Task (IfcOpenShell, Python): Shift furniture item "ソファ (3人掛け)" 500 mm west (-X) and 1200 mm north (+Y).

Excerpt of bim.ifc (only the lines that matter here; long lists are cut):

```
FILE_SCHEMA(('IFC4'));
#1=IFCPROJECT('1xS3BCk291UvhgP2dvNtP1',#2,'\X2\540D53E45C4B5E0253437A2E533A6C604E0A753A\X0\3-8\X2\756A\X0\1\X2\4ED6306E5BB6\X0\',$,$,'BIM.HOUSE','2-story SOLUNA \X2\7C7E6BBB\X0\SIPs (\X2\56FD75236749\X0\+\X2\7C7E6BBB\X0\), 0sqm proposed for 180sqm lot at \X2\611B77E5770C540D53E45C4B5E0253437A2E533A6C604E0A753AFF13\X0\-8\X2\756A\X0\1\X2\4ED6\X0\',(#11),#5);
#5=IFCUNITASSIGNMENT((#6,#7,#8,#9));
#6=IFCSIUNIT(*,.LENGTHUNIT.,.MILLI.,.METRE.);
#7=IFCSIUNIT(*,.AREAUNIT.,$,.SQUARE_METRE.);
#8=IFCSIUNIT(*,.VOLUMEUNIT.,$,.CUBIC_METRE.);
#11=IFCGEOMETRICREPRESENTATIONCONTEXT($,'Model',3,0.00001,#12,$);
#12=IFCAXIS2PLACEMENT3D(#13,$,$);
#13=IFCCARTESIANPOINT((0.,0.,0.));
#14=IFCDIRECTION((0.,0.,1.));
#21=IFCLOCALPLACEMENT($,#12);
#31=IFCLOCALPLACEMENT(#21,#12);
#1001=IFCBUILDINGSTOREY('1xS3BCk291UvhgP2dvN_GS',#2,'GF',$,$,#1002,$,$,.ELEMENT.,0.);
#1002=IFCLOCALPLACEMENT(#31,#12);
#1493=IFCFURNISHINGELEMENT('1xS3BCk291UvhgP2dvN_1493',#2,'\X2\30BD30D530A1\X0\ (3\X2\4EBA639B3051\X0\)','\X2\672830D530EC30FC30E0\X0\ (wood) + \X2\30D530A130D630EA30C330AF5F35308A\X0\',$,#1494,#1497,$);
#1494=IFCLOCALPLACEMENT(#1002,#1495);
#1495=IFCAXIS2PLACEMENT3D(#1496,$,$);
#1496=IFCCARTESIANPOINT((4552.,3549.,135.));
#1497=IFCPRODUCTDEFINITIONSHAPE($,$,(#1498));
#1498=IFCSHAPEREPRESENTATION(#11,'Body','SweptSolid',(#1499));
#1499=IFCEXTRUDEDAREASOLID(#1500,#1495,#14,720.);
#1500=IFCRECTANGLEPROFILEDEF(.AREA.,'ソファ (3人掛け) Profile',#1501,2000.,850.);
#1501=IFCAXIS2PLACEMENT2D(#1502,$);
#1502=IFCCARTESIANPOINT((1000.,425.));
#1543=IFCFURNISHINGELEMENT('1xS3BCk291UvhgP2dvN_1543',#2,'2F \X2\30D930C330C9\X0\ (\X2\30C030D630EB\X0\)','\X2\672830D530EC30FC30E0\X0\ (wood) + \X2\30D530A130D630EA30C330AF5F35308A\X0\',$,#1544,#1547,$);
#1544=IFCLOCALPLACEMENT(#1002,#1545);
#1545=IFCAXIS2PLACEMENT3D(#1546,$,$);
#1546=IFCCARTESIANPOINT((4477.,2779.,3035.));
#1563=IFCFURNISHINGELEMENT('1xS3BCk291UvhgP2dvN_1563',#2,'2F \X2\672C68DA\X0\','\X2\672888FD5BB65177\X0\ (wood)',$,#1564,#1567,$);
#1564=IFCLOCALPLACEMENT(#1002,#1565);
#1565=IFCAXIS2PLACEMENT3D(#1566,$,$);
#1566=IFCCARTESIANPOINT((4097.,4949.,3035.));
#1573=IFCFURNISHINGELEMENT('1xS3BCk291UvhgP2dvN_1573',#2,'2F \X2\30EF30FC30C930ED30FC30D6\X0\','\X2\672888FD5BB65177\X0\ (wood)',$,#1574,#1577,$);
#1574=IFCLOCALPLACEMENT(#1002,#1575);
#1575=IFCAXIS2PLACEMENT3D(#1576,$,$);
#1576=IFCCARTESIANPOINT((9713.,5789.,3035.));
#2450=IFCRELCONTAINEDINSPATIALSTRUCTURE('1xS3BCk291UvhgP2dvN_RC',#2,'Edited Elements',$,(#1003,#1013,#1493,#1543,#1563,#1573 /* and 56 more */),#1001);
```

```python
import ifcopenshell
import ifcopenshell.api.geometry
import ifcopenshell.util.placement
import ifcopenshell.util.unit

model = ifcopenshell.open("bim.ifc")
unit_scale = ifcopenshell.util.unit.calculate_unit_scale(model)

item = model.by_guid("1xS3BCk291UvhgP2dvN_1493")
matrix = ifcopenshell.util.placement.get_local_placement(item.ObjectPlacement)
matrix[0, 3] -= 0.5 / unit_scale
matrix[1, 3] += 1.2 / unit_scale
ifcopenshell.api.geometry.edit_object_placement(model, product=item, matrix=matrix, is_si=False)

print(ifcopenshell.util.placement.get_local_placement(item.ObjectPlacement).round(3) + 0.0)

model.write("bim_updated.ifc")
```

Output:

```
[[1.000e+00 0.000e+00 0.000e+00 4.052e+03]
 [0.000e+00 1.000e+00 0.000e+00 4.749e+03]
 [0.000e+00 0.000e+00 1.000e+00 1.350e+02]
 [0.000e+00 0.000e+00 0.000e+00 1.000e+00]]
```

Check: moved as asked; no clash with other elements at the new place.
